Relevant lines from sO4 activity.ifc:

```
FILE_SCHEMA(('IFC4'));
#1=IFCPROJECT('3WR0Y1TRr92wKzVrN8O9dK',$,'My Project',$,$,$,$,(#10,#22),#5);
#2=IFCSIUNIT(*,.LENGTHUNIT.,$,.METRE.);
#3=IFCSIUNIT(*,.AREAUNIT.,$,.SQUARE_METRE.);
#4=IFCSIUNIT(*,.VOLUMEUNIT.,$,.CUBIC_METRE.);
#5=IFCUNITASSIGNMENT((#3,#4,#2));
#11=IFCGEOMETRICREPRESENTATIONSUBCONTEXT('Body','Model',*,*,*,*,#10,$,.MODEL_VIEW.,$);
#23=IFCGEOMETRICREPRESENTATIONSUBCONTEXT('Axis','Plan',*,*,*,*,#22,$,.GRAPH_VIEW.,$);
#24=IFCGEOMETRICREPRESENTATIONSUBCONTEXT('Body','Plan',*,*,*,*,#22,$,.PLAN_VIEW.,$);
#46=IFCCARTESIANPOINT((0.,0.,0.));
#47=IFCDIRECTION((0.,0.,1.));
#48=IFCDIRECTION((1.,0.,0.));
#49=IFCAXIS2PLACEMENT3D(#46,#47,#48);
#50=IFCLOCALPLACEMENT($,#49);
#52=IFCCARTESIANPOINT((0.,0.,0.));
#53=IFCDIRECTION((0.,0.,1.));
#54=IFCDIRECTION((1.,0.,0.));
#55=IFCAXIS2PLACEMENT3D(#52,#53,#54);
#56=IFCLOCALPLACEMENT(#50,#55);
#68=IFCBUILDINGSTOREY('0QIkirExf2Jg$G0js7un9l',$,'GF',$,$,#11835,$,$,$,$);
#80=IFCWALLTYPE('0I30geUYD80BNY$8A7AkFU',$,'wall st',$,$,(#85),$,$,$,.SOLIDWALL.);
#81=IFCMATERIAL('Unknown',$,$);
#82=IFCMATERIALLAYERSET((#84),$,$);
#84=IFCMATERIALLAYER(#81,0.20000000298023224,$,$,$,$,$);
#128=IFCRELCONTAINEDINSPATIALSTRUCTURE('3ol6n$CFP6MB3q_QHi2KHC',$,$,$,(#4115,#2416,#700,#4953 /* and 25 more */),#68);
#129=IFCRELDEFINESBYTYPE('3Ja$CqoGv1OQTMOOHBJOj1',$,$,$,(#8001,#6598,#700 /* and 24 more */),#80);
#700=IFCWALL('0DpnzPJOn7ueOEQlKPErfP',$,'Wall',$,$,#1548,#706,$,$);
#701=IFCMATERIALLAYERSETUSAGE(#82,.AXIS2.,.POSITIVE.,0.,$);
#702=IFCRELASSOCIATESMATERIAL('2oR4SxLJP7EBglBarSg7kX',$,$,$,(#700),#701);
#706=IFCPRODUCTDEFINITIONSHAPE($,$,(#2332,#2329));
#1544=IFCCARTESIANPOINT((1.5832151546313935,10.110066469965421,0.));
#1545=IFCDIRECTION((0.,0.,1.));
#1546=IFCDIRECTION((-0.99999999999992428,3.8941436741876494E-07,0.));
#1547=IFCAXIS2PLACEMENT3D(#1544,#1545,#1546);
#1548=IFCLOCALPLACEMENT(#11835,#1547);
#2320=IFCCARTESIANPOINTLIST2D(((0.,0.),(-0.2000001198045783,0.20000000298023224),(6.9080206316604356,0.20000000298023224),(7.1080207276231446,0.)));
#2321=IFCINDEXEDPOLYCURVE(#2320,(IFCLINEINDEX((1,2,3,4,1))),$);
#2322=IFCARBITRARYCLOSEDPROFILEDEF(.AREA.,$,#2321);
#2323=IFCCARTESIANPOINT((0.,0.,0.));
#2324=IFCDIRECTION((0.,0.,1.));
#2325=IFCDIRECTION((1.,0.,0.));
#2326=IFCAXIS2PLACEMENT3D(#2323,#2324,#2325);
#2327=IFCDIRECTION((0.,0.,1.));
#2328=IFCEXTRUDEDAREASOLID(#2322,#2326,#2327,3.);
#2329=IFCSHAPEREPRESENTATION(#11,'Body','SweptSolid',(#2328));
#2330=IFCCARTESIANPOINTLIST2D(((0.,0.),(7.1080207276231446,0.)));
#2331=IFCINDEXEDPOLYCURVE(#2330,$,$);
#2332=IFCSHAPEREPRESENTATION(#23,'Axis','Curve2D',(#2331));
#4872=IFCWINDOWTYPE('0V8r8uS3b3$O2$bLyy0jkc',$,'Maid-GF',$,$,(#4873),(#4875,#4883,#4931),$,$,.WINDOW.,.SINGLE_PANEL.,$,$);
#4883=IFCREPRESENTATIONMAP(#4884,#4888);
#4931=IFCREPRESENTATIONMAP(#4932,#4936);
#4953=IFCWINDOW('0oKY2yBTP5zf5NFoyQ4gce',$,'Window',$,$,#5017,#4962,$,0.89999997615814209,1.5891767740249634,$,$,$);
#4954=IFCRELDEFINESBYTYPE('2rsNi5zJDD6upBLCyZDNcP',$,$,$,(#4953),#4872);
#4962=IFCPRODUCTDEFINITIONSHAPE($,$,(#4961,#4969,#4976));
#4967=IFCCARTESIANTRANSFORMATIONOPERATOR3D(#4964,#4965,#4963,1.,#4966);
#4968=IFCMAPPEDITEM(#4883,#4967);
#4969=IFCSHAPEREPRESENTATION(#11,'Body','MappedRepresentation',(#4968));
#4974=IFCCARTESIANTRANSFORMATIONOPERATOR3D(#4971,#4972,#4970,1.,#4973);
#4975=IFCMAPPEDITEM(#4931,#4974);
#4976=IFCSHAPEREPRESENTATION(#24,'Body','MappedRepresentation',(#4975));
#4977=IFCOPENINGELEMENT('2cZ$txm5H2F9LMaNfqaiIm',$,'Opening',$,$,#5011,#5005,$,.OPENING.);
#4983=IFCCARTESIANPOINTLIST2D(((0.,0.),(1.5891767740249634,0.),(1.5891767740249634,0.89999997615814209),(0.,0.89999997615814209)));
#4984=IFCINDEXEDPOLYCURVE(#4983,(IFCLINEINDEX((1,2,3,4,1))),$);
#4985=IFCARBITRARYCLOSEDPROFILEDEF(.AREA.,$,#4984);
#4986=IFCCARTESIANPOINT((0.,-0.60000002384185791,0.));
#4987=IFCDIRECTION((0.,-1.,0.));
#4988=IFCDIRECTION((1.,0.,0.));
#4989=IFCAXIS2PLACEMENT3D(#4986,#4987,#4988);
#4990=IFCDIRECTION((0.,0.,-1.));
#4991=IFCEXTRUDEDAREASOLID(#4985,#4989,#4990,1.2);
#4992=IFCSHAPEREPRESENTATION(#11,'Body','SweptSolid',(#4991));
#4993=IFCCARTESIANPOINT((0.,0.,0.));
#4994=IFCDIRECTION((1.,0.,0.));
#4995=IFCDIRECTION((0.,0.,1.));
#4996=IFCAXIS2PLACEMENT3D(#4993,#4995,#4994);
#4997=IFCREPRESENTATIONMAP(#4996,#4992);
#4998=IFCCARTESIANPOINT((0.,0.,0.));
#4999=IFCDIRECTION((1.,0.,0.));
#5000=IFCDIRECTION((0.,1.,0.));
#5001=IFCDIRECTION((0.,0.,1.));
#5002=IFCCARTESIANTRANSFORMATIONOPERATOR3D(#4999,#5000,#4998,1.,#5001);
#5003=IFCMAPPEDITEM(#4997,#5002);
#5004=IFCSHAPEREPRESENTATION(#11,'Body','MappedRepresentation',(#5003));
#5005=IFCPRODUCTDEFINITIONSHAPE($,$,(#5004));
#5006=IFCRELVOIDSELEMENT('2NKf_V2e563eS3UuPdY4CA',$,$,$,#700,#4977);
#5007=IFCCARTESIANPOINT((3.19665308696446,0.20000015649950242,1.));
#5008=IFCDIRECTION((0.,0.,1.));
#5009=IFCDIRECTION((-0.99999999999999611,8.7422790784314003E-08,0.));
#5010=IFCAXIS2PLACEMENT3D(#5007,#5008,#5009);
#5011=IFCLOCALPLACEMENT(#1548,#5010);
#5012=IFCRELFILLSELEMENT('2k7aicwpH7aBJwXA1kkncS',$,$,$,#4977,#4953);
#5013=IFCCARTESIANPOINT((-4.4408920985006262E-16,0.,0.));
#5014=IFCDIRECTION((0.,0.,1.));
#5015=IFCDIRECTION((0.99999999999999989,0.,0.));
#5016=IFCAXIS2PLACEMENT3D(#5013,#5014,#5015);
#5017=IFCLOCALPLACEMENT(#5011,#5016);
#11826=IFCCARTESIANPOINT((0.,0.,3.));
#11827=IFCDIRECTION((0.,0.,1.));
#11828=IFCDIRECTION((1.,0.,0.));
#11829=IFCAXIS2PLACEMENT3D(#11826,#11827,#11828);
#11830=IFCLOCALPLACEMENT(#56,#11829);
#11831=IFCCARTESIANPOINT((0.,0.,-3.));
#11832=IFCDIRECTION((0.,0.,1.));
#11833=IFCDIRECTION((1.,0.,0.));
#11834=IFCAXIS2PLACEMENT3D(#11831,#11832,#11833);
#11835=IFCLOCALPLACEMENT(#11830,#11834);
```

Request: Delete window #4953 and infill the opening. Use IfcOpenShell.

```python
import ifcopenshell
import ifcopenshell.api.feature
import ifcopenshell.api.root
import ifcopenshell.geom
import ifcopenshell.util.shape

model = ifcopenshell.open("sO4 activity.ifc")
settings = ifcopenshell.geom.settings()


def volume(element):
    """Net volume in cubic metres, openings subtracted."""
    shape = ifcopenshell.geom.create_shape(settings, element)
    return ifcopenshell.util.shape.get_volume(shape.geometry)


window = model.by_id(4953)
opening = window.FillsVoids[0].RelatingOpeningElement
wall = opening.VoidsElements[0].RelatingBuildingElement
before = volume(wall)

ifcopenshell.api.root.remove_product(model, product=window)
ifcopenshell.api.feature.remove_feature(model, feature=opening)

after = volume(wall)

print(f"wall volume {before:.3f} -> {after:.3f} m3")

model.write("sO4 activity_rev.ifc")
```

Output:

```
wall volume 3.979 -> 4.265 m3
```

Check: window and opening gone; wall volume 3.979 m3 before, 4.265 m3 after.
